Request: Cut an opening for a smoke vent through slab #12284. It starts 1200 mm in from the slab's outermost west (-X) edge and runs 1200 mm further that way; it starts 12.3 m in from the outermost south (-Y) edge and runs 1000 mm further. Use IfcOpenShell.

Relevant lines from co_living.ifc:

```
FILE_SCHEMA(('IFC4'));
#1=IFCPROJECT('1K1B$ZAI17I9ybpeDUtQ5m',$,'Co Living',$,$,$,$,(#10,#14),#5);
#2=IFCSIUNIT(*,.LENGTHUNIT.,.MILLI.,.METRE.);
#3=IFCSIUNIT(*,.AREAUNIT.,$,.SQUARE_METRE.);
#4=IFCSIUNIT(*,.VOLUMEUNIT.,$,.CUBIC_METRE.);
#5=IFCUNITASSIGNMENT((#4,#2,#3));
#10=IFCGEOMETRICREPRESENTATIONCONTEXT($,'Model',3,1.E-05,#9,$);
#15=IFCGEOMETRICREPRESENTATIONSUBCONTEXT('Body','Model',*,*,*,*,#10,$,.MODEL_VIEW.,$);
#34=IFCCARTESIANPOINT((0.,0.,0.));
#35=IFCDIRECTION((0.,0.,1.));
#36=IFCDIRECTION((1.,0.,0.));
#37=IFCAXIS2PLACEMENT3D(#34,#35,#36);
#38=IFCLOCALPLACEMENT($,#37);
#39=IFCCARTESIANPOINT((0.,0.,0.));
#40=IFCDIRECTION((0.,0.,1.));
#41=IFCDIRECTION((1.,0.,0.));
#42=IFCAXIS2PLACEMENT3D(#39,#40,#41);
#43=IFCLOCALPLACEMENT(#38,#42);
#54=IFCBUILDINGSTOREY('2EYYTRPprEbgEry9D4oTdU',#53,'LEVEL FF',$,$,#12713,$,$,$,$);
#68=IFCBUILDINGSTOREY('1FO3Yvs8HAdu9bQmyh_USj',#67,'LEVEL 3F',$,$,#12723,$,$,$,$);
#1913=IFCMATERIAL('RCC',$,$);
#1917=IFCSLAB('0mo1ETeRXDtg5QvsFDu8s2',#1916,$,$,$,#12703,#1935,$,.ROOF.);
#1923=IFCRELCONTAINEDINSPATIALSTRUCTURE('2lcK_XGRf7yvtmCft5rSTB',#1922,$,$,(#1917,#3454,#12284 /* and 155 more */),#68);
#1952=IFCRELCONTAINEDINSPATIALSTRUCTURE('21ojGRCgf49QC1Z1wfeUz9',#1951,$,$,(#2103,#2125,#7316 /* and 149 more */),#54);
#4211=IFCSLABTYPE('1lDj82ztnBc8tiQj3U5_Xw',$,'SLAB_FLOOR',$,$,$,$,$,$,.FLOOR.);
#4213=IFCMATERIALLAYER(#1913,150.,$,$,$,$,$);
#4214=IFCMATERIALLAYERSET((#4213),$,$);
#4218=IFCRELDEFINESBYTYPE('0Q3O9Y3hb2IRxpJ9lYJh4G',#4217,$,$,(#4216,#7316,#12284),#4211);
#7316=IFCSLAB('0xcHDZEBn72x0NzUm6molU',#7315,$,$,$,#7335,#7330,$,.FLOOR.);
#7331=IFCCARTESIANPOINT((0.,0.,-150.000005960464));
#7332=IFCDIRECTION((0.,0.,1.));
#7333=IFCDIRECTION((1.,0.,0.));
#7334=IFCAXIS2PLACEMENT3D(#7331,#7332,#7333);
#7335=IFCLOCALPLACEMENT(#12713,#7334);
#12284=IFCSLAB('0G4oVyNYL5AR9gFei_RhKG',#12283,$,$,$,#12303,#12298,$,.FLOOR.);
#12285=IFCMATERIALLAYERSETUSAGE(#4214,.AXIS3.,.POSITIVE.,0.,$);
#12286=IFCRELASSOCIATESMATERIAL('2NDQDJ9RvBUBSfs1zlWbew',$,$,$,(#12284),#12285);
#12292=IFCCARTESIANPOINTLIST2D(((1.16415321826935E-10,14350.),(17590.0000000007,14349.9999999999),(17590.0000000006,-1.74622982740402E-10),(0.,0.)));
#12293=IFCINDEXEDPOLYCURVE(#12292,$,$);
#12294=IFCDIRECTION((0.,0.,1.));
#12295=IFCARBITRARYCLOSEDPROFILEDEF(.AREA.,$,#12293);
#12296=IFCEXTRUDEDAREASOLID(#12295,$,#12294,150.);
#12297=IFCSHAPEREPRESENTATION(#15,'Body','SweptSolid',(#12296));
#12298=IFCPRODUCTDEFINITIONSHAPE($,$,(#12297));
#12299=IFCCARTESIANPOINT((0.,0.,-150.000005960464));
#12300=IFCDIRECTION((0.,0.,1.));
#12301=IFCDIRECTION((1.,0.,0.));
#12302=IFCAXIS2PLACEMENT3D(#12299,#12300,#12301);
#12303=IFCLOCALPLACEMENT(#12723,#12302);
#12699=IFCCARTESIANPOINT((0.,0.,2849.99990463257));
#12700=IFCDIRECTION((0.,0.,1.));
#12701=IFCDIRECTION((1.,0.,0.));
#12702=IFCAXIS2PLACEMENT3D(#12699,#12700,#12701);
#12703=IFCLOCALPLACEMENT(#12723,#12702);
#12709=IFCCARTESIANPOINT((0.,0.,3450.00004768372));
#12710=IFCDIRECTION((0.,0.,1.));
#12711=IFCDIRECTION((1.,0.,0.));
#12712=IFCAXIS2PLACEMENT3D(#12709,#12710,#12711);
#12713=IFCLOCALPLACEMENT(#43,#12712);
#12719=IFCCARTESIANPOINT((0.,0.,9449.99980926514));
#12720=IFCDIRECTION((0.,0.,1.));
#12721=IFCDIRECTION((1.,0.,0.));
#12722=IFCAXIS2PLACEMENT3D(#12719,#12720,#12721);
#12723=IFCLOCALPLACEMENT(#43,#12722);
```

```python
import numpy as np
import ifcopenshell
import ifcopenshell.api.feature
import ifcopenshell.api.geometry
import ifcopenshell.api.root
import ifcopenshell.geom
import ifcopenshell.util.placement
import ifcopenshell.util.representation
import ifcopenshell.util.shape
import ifcopenshell.util.unit

model = ifcopenshell.open("co_living.ifc")
unit_scale = ifcopenshell.util.unit.calculate_unit_scale(model)
settings = ifcopenshell.geom.settings()


def volume(element):
    """Net volume in cubic metres, openings subtracted."""
    shape = ifcopenshell.geom.create_shape(settings, element)
    return ifcopenshell.util.shape.get_volume(shape.geometry)


slab = model.by_guid("0G4oVyNYL5AR9gFei_RhKG")
before = volume(slab)

# Extent in the slab's own axes, in metres. The edges named are its -X and -Y sides.
slab_shape = ifcopenshell.geom.create_shape(settings, slab)
vertices = ifcopenshell.util.shape.get_vertices(slab_shape.geometry)
x_min, y_min, bottom = vertices.min(axis=0)
top = vertices[:, 2].max()

opening = ifcopenshell.api.root.create_entity(model, ifc_class="IfcOpeningElement", name="Smoke vent opening", predefined_type="OPENING")
context = ifcopenshell.util.representation.get_context(model, "Model", "Body", "MODEL_VIEW")
width, depth = 1.2, 1
outline = [(0.0, 0.0), (width, 0.0), (width, depth), (0.0, depth), (0.0, 0.0)]
# Overshoot both faces by 50 mm so the cut is clean.
shape = ifcopenshell.api.geometry.add_slab_representation(
    model, context=context, depth=top - bottom + 0.1, polyline=outline
)
ifcopenshell.api.geometry.assign_representation(model, product=opening, representation=shape)

matrix = ifcopenshell.util.placement.get_local_placement(slab.ObjectPlacement)
matrix[:, 3] = matrix @ np.append(np.array([x_min + 1.2, y_min + 12.3, bottom - 0.05]) / unit_scale, 1.0)
ifcopenshell.api.geometry.edit_object_placement(model, product=opening, matrix=matrix, is_si=False)
ifcopenshell.api.feature.add_feature(model, feature=opening, element=slab)

after = volume(slab)

print(f"slab volume {before:.3f} -> {after:.3f} m3")

model.write("co_living_edited.ifc")
```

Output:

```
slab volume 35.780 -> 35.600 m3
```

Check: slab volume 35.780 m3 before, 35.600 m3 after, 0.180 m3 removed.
